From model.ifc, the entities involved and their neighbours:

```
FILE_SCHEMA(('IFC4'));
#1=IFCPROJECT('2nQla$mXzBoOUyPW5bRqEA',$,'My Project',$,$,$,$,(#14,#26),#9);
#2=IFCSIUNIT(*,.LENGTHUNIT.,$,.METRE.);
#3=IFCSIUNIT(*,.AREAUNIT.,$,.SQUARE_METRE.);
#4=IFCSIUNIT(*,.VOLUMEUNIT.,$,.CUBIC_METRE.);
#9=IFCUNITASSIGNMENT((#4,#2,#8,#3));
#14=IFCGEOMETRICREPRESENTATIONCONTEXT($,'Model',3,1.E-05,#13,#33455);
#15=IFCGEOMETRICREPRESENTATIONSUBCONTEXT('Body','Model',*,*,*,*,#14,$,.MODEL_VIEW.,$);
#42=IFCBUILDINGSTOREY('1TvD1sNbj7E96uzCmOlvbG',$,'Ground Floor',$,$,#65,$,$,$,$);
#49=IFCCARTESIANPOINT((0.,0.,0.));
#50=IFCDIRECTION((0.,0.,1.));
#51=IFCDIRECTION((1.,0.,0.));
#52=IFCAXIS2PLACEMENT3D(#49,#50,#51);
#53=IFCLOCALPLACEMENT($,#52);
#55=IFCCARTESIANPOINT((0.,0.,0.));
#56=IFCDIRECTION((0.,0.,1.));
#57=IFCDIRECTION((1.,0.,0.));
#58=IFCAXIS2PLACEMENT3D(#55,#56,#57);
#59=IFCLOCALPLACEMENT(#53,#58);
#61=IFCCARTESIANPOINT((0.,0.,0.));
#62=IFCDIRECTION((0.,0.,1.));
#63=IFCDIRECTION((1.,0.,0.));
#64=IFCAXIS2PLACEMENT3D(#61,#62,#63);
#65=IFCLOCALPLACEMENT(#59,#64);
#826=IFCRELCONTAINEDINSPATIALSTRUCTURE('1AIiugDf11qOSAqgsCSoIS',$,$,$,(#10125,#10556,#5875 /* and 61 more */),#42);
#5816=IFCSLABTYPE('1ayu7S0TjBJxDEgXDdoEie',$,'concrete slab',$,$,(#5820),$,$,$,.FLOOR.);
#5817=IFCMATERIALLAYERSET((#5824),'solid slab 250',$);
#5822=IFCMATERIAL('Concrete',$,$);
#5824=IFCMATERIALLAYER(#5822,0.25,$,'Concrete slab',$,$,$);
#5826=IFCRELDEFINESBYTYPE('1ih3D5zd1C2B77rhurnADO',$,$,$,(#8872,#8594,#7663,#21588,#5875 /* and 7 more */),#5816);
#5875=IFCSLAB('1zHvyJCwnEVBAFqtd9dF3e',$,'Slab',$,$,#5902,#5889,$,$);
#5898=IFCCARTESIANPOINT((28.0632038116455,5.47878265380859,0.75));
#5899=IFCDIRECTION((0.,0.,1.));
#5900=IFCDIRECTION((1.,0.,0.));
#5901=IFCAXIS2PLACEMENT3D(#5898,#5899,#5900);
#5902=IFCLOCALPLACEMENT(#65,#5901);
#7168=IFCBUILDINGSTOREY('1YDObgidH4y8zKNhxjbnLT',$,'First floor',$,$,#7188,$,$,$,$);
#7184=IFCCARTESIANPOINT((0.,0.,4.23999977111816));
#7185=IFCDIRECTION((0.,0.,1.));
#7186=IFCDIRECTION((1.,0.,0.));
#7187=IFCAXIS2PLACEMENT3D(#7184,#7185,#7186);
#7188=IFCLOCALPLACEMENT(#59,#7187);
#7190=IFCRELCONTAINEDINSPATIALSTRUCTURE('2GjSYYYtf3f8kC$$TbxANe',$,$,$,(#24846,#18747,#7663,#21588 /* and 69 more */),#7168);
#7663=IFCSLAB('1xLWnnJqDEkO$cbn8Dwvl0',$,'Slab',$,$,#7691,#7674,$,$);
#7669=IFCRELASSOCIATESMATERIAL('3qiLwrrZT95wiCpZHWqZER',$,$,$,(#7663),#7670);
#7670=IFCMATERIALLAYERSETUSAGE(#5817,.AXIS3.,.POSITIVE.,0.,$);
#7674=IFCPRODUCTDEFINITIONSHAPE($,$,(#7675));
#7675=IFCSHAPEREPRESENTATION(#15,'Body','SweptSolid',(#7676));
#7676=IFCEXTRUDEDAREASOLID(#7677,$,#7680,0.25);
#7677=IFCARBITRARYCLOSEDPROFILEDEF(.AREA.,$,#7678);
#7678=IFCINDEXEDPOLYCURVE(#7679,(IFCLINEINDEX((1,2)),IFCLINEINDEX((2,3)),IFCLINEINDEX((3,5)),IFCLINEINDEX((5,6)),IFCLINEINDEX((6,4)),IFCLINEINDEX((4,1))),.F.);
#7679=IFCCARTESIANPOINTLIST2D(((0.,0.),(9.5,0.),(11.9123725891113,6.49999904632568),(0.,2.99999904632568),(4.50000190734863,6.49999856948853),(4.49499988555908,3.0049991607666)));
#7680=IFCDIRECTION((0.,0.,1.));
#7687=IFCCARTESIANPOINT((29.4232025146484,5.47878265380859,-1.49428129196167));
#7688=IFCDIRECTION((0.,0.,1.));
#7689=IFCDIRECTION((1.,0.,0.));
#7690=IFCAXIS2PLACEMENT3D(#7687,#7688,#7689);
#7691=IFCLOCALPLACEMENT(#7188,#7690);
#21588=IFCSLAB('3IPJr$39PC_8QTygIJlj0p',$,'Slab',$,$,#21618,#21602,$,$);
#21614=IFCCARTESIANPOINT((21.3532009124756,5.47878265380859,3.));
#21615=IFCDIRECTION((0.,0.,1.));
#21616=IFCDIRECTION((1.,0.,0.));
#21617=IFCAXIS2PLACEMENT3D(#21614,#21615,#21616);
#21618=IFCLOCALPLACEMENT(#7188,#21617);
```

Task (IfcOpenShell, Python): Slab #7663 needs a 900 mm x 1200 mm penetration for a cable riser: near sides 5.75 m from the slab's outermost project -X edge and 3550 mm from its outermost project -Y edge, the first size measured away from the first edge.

```python
import numpy as np
import ifcopenshell
import ifcopenshell.api.feature
import ifcopenshell.api.geometry
import ifcopenshell.api.root
import ifcopenshell.geom
import ifcopenshell.util.placement
import ifcopenshell.util.representation
import ifcopenshell.util.shape
import ifcopenshell.util.unit

model = ifcopenshell.open("model.ifc")
unit_scale = ifcopenshell.util.unit.calculate_unit_scale(model)
settings = ifcopenshell.geom.settings()


def volume(element):
    """Net volume in cubic metres, openings subtracted."""
    shape = ifcopenshell.geom.create_shape(settings, element)
    return ifcopenshell.util.shape.get_volume(shape.geometry)


slab = model.by_guid("1xLWnnJqDEkO$cbn8Dwvl0")
before = volume(slab)

# Extent in the slab's own axes, in metres. The edges named are its -X and -Y sides.
slab_shape = ifcopenshell.geom.create_shape(settings, slab)
vertices = ifcopenshell.util.shape.get_vertices(slab_shape.geometry)
x_min, y_min, bottom = vertices.min(axis=0)
top = vertices[:, 2].max()

opening = ifcopenshell.api.root.create_entity(model, ifc_class="IfcOpeningElement", name="Cable riser opening", predefined_type="OPENING")
context = ifcopenshell.util.representation.get_context(model, "Model", "Body", "MODEL_VIEW")
width, depth = 0.9, 1.2
outline = [(0.0, 0.0), (width, 0.0), (width, depth), (0.0, depth), (0.0, 0.0)]
# Overshoot both faces by 50 mm so the cut is clean.
shape = ifcopenshell.api.geometry.add_slab_representation(
    model, context=context, depth=top - bottom + 0.1, polyline=outline
)
ifcopenshell.api.geometry.assign_representation(model, product=opening, representation=shape)

matrix = ifcopenshell.util.placement.get_local_placement(slab.ObjectPlacement)
matrix[:, 3] = matrix @ np.append(np.array([x_min + 5.75, y_min + 3.55, bottom - 0.05]) / unit_scale, 1.0)
ifcopenshell.api.geometry.edit_object_placement(model, product=opening, matrix=matrix, is_si=False)
ifcopenshell.api.feature.add_feature(model, feature=opening, element=slab)

after = volume(slab)

print(f"slab volume {before:.3f} -> {after:.3f} m3")

model.write("model_rev.ifc")
```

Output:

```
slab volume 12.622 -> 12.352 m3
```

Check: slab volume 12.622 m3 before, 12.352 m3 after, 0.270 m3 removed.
